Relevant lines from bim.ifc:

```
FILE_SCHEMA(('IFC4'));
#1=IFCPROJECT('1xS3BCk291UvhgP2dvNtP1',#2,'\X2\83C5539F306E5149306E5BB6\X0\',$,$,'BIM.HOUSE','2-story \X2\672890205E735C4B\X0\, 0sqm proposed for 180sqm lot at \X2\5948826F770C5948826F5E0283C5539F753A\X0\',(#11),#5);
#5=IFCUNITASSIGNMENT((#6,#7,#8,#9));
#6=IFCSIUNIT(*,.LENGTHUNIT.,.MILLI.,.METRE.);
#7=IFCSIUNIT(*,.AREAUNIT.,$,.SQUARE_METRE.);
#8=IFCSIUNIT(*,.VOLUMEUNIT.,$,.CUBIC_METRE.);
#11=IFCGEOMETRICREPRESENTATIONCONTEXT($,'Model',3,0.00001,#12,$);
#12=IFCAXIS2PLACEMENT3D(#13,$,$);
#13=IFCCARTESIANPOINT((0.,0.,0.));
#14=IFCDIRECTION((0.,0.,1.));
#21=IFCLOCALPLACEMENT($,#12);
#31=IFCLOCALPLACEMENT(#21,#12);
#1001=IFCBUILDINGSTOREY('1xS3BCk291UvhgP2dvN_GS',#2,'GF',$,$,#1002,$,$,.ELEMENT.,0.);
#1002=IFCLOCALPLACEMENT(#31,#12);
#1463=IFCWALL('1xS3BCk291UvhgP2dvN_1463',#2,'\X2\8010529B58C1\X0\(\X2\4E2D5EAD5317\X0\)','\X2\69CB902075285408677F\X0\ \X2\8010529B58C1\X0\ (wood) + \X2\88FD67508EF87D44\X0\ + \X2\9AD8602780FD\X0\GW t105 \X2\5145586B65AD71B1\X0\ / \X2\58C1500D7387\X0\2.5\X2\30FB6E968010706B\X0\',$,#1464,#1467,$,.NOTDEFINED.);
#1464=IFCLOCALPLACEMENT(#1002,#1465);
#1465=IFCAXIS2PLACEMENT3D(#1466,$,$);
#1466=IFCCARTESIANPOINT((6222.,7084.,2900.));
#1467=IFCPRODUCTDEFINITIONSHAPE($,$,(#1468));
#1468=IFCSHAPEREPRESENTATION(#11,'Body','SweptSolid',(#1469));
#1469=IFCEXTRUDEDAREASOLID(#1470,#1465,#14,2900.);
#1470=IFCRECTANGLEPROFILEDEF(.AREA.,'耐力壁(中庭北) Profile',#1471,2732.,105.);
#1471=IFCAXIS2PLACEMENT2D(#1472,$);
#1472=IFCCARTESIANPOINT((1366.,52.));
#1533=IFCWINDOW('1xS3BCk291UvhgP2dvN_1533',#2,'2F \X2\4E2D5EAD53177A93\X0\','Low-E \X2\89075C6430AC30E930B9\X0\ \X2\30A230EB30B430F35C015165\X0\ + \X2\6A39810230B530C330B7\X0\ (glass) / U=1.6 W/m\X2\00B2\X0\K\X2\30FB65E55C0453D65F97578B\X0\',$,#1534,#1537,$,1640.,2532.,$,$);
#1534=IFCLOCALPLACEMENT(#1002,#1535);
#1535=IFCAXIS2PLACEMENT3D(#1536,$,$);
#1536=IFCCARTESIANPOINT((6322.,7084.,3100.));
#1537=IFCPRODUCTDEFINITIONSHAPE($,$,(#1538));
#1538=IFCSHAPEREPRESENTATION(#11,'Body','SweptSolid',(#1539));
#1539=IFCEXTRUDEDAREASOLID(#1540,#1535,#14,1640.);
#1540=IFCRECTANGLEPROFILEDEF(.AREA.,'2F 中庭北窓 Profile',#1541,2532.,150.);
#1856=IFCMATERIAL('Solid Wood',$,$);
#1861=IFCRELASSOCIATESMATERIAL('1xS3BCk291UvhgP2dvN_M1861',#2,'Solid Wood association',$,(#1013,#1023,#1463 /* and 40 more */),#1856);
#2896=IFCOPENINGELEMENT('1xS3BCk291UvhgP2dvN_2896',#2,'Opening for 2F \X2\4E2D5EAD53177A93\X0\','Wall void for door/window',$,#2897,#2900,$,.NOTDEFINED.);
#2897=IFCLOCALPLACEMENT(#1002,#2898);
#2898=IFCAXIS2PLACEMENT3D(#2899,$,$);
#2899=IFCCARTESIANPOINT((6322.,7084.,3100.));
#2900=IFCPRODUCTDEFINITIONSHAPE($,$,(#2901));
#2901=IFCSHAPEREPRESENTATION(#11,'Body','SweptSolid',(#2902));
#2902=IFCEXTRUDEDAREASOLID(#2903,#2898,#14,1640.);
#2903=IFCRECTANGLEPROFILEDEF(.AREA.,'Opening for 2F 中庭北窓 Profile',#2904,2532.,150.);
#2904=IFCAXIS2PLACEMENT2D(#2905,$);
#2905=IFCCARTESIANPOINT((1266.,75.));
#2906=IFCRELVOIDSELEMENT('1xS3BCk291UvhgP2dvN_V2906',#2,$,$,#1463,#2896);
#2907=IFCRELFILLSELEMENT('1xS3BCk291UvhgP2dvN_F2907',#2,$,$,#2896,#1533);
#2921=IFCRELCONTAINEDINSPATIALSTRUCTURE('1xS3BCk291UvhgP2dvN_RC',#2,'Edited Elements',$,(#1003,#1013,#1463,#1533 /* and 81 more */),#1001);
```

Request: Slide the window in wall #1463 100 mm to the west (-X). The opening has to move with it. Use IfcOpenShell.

```python
import ifcopenshell
import ifcopenshell.api.geometry
import ifcopenshell.util.placement
import ifcopenshell.util.unit

model = ifcopenshell.open("bim.ifc")
unit_scale = ifcopenshell.util.unit.calculate_unit_scale(model)

window = model.by_guid("1xS3BCk291UvhgP2dvN_1533")
opening = window.FillsVoids[0].RelatingOpeningElement
wall = opening.VoidsElements[0].RelatingBuildingElement

wall_matrix = ifcopenshell.util.placement.get_local_placement(wall.ObjectPlacement)
shift = wall_matrix[:3, 0] * -0.1 / unit_scale
before = ifcopenshell.util.placement.get_local_placement(window.ObjectPlacement)[:3, 3].copy()

# The window is not placed relative to its opening, so move both.
for product in (opening, window):
    matrix = ifcopenshell.util.placement.get_local_placement(product.ObjectPlacement)
    matrix[:3, 3] += shift
    ifcopenshell.api.geometry.edit_object_placement(model, product=product, matrix=matrix, is_si=False)

after = ifcopenshell.util.placement.get_local_placement(window.ObjectPlacement)[:3, 3]
print("window moved by", (after - before).round(3) + 0.0)

model.write("bim_updated.ifc")
```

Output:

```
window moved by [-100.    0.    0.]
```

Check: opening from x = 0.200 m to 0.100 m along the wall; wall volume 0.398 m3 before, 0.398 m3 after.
